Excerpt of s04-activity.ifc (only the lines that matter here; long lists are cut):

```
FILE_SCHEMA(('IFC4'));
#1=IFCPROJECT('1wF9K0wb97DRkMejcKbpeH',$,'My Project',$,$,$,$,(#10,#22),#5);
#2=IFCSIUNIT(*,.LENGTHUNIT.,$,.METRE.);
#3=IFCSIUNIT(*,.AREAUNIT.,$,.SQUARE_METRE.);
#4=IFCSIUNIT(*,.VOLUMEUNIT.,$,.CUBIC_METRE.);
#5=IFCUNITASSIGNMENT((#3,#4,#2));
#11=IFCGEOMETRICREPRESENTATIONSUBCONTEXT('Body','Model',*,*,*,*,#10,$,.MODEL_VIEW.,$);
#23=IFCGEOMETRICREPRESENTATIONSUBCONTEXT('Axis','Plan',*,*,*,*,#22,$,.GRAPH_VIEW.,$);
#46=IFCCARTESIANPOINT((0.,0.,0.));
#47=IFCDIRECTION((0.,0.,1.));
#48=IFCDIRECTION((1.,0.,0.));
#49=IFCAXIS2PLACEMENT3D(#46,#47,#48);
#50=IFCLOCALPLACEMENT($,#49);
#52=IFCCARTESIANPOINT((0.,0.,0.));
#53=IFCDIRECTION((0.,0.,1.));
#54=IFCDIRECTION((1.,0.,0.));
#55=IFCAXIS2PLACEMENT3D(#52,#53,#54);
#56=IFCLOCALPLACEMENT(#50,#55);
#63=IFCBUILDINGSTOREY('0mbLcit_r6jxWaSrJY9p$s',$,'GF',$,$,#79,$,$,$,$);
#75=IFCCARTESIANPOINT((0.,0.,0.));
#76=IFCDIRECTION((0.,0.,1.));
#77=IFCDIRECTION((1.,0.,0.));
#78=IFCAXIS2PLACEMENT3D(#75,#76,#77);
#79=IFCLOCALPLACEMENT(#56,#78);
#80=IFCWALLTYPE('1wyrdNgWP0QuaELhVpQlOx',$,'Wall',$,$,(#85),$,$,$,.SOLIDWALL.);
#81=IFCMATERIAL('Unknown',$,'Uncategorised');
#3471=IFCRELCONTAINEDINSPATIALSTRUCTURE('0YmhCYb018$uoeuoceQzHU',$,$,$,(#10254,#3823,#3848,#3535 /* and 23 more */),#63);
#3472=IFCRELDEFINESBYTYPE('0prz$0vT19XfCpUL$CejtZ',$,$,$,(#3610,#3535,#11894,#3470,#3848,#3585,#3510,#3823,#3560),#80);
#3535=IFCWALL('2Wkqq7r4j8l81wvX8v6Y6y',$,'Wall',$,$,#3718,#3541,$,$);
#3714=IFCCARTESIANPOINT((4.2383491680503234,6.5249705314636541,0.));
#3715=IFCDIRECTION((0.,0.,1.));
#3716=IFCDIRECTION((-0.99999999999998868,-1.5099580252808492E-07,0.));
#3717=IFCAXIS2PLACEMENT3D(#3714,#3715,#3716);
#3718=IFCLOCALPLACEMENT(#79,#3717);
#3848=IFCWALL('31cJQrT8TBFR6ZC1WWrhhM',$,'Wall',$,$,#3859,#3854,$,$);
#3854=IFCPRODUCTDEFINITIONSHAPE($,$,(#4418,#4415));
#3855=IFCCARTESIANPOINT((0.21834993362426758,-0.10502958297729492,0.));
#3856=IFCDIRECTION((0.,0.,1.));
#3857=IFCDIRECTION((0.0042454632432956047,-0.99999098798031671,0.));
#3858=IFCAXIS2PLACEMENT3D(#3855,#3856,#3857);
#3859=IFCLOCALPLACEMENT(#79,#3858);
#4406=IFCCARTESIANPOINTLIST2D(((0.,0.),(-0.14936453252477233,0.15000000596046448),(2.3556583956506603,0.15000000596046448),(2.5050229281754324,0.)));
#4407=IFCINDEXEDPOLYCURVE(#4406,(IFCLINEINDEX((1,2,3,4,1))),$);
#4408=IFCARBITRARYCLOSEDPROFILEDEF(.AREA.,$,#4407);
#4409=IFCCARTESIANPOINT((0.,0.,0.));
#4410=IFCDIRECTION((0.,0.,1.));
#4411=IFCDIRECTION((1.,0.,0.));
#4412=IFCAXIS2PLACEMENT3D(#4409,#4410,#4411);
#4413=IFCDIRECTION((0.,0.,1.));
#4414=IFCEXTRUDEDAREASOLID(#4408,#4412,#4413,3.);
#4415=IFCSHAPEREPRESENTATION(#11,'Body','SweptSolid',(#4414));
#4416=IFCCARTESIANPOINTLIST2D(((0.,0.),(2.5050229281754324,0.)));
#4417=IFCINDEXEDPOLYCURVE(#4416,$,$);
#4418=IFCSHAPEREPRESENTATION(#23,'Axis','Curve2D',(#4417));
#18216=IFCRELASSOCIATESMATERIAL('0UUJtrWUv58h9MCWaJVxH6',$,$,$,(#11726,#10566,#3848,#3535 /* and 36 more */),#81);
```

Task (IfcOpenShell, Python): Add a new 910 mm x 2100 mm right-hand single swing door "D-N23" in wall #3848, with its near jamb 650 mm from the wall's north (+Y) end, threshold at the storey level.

```python
import numpy as np
import ifcopenshell
import ifcopenshell.api.feature
import ifcopenshell.api.geometry
import ifcopenshell.api.root
import ifcopenshell.api.spatial
import ifcopenshell.geom
import ifcopenshell.util.element
import ifcopenshell.util.placement
import ifcopenshell.util.representation
import ifcopenshell.util.shape
import ifcopenshell.util.unit

model = ifcopenshell.open("s04-activity.ifc")
unit_scale = ifcopenshell.util.unit.calculate_unit_scale(model)
settings = ifcopenshell.geom.settings()


def volume(element):
    """Net volume in cubic metres, openings subtracted."""
    shape = ifcopenshell.geom.create_shape(settings, element)
    return ifcopenshell.util.shape.get_volume(shape.geometry)


wall = model.by_guid("31cJQrT8TBFR6ZC1WWrhhM")
storey = ifcopenshell.util.element.get_container(wall, ifc_class="IfcBuildingStorey")
context = ifcopenshell.util.representation.get_context(model, "Model", "Body", "MODEL_VIEW")
before = volume(wall)

width, height, from_end, sill = 0.91, 2.1, 0.65, 0.0  # metres

# The wall runs along its own X axis, and the end named is its -X end.
wall_shape = ifcopenshell.geom.create_shape(settings, wall)
x, y, z = ifcopenshell.util.shape.get_vertices(wall_shape.geometry).T
start = x.min() + from_end
face, thickness = float(y.min()), float(y.max() - y.min())
wall_matrix = ifcopenshell.util.placement.get_local_placement(wall.ObjectPlacement)
level = ifcopenshell.util.placement.get_local_placement(storey.ObjectPlacement)[2, 3]


def in_wall(x, y):
    """Placement at x, y metres in the wall's axes, at sill height."""
    matrix = wall_matrix.copy()
    matrix[:, 3] = wall_matrix @ np.array([x / unit_scale, y / unit_scale, 0.0, 1.0])
    matrix[2, 3] = level + sill / unit_scale
    return matrix


# Opening: a box that overshoots both wall faces by 50 mm.
opening = ifcopenshell.api.root.create_entity(model, ifc_class="IfcOpeningElement", predefined_type="OPENING")
box = ifcopenshell.api.geometry.add_wall_representation(
    model, context=context, length=width, height=height, thickness=thickness + 0.1
)
ifcopenshell.api.geometry.assign_representation(model, product=opening, representation=box)
ifcopenshell.api.geometry.edit_object_placement(model, product=opening, matrix=in_wall(start, face - 0.05), is_si=False)
ifcopenshell.api.feature.add_feature(model, feature=opening, element=wall)

door = ifcopenshell.api.root.create_entity(model, ifc_class="IfcDoor", name="D-N23", predefined_type="DOOR")
door.OverallWidth, door.OverallHeight = width / unit_scale, height / unit_scale
door.OperationType = "SINGLE_SWING_RIGHT"
body = ifcopenshell.api.geometry.add_door_representation(
    model,
    context=context,
    overall_width=door.OverallWidth,
    overall_height=door.OverallHeight,
    operation_type="SINGLE_SWING_RIGHT",
    lining_properties={"LiningDepth": thickness / unit_scale, "ThresholdDepth": thickness / unit_scale},
)
ifcopenshell.api.geometry.assign_representation(model, product=door, representation=body)
ifcopenshell.api.spatial.assign_container(model, products=[door], relating_structure=storey)
ifcopenshell.api.feature.add_filling(model, opening=opening, element=door)

# The lining spans the wall, so the door starts at the wall face.
ifcopenshell.api.geometry.edit_object_placement(model, product=door, matrix=in_wall(start, face), is_si=False)

after = volume(wall)

print(f"wall volume {before:.3f} -> {after:.3f} m3")

model.write("s04-activity_v2.ifc")
```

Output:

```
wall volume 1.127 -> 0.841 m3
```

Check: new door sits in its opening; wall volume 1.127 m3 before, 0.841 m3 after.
